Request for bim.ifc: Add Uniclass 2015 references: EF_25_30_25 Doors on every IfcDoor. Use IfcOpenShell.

First a look at what the model holds.

```python
import ifcopenshell

model = ifcopenshell.open("bim.ifc")
print(model.schema)
print("classifications:", [c.Name for c in model.by_type("IfcClassification")])
for ifc_class in ("IfcDoor", "IfcRoof", "IfcStair", "IfcWall", "IfcWindow"):
    print(ifc_class, len(model.by_type(ifc_class)))
```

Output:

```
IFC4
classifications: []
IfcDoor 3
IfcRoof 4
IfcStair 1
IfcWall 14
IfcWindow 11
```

```python
import ifcopenshell
import ifcopenshell.api.classification

model = ifcopenshell.open("bim.ifc")

system = ifcopenshell.api.classification.add_classification(model, classification="Uniclass 2015")

codes = {
    "IfcDoor": ("EF_25_30_25", "Doors"),
}
for ifc_class, (code, name) in codes.items():
    products = model.by_type(ifc_class)
    ifcopenshell.api.classification.add_reference(
        model, products=products, classification=system, identification=code, name=name
    )
    print(code, len(products))

model.write("bim_edited.ifc")
```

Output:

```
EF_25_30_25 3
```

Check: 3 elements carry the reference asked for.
